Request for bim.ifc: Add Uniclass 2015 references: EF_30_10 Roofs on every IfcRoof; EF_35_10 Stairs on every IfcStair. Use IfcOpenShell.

First a look at what the model holds.

```python
import ifcopenshell

model = ifcopenshell.open("bim.ifc")
print(model.schema)
print("classifications:", [c.Name for c in model.by_type("IfcClassification")])
for ifc_class in ("IfcDoor", "IfcRoof", "IfcStair", "IfcWall", "IfcWindow"):
    print(ifc_class, len(model.by_type(ifc_class)))
```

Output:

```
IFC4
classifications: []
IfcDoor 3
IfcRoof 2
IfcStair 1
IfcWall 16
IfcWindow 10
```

```python
import ifcopenshell
import ifcopenshell.api.classification

model = ifcopenshell.open("bim.ifc")

system = ifcopenshell.api.classification.add_classification(model, classification="Uniclass 2015")

codes = {
    "IfcRoof": ("EF_30_10", "Roofs"),
    "IfcStair": ("EF_35_10", "Stairs"),
}
for ifc_class, (code, name) in codes.items():
    products = model.by_type(ifc_class)
    ifcopenshell.api.classification.add_reference(
        model, products=products, classification=system, identification=code, name=name
    )
    print(code, len(products))

model.write("bim_v2.ifc")
```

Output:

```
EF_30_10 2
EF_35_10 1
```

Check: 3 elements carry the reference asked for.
